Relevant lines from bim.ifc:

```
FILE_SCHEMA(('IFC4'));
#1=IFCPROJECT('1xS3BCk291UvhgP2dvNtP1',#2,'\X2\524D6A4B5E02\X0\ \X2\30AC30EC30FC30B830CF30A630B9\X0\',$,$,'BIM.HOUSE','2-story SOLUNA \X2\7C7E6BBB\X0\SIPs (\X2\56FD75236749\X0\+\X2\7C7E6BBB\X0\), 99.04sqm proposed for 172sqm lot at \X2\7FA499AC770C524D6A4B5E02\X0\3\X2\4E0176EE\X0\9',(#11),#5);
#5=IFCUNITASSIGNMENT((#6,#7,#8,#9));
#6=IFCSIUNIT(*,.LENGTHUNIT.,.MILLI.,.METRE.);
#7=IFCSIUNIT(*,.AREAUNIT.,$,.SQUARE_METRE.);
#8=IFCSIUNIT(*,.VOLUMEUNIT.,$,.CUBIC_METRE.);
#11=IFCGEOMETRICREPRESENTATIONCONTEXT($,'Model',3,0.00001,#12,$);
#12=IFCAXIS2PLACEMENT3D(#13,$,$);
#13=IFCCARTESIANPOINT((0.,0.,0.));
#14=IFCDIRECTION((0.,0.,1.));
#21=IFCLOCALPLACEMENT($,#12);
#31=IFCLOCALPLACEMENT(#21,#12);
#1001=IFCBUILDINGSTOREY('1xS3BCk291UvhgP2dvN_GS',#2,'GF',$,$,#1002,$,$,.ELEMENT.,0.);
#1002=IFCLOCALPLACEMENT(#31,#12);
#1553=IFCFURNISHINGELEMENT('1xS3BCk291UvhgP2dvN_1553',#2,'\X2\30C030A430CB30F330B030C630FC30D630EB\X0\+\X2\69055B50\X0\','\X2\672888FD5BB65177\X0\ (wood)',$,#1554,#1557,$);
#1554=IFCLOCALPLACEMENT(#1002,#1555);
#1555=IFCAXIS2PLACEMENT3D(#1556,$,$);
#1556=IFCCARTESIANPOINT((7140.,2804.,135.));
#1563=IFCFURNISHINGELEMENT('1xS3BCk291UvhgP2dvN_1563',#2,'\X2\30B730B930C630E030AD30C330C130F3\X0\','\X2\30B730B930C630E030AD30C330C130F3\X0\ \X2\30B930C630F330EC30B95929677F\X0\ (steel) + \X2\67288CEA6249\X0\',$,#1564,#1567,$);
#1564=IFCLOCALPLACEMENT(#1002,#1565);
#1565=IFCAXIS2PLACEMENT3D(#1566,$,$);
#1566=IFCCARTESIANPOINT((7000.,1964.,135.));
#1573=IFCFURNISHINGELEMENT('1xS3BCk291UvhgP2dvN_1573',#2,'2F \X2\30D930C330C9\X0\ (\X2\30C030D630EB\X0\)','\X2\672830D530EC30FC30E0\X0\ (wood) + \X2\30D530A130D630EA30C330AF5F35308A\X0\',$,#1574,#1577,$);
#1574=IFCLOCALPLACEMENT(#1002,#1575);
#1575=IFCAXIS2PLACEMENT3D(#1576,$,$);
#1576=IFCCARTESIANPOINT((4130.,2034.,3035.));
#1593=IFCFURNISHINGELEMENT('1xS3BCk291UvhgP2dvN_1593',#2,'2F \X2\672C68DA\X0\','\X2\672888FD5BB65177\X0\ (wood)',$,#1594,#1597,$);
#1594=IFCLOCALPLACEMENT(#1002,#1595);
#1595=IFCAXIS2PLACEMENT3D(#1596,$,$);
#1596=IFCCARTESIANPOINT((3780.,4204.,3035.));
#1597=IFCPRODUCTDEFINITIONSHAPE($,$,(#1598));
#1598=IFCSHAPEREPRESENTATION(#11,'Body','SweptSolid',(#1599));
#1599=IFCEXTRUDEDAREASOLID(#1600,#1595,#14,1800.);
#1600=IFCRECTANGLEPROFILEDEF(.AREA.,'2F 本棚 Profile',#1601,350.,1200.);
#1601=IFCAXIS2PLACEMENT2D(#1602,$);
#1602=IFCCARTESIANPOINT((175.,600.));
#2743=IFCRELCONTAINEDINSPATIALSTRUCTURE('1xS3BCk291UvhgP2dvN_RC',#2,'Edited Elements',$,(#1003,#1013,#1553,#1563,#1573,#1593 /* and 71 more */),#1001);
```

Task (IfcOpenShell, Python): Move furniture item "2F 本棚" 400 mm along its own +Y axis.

```python
import ifcopenshell
import ifcopenshell.api.geometry
import ifcopenshell.util.placement
import ifcopenshell.util.unit

model = ifcopenshell.open("bim.ifc")
unit_scale = ifcopenshell.util.unit.calculate_unit_scale(model)

item = model.by_id(1593)
matrix = ifcopenshell.util.placement.get_local_placement(item.ObjectPlacement)
matrix[:3, 3] += matrix[:3, 1] * 0.4 / unit_scale
ifcopenshell.api.geometry.edit_object_placement(model, product=item, matrix=matrix, is_si=False)

print(ifcopenshell.util.placement.get_local_placement(item.ObjectPlacement).round(3) + 0.0)

model.write("bim_rev.ifc")
```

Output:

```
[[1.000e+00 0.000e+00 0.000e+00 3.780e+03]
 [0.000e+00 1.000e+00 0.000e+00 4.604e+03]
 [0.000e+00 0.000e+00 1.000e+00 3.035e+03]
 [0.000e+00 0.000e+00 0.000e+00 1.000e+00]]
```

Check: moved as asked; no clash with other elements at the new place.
